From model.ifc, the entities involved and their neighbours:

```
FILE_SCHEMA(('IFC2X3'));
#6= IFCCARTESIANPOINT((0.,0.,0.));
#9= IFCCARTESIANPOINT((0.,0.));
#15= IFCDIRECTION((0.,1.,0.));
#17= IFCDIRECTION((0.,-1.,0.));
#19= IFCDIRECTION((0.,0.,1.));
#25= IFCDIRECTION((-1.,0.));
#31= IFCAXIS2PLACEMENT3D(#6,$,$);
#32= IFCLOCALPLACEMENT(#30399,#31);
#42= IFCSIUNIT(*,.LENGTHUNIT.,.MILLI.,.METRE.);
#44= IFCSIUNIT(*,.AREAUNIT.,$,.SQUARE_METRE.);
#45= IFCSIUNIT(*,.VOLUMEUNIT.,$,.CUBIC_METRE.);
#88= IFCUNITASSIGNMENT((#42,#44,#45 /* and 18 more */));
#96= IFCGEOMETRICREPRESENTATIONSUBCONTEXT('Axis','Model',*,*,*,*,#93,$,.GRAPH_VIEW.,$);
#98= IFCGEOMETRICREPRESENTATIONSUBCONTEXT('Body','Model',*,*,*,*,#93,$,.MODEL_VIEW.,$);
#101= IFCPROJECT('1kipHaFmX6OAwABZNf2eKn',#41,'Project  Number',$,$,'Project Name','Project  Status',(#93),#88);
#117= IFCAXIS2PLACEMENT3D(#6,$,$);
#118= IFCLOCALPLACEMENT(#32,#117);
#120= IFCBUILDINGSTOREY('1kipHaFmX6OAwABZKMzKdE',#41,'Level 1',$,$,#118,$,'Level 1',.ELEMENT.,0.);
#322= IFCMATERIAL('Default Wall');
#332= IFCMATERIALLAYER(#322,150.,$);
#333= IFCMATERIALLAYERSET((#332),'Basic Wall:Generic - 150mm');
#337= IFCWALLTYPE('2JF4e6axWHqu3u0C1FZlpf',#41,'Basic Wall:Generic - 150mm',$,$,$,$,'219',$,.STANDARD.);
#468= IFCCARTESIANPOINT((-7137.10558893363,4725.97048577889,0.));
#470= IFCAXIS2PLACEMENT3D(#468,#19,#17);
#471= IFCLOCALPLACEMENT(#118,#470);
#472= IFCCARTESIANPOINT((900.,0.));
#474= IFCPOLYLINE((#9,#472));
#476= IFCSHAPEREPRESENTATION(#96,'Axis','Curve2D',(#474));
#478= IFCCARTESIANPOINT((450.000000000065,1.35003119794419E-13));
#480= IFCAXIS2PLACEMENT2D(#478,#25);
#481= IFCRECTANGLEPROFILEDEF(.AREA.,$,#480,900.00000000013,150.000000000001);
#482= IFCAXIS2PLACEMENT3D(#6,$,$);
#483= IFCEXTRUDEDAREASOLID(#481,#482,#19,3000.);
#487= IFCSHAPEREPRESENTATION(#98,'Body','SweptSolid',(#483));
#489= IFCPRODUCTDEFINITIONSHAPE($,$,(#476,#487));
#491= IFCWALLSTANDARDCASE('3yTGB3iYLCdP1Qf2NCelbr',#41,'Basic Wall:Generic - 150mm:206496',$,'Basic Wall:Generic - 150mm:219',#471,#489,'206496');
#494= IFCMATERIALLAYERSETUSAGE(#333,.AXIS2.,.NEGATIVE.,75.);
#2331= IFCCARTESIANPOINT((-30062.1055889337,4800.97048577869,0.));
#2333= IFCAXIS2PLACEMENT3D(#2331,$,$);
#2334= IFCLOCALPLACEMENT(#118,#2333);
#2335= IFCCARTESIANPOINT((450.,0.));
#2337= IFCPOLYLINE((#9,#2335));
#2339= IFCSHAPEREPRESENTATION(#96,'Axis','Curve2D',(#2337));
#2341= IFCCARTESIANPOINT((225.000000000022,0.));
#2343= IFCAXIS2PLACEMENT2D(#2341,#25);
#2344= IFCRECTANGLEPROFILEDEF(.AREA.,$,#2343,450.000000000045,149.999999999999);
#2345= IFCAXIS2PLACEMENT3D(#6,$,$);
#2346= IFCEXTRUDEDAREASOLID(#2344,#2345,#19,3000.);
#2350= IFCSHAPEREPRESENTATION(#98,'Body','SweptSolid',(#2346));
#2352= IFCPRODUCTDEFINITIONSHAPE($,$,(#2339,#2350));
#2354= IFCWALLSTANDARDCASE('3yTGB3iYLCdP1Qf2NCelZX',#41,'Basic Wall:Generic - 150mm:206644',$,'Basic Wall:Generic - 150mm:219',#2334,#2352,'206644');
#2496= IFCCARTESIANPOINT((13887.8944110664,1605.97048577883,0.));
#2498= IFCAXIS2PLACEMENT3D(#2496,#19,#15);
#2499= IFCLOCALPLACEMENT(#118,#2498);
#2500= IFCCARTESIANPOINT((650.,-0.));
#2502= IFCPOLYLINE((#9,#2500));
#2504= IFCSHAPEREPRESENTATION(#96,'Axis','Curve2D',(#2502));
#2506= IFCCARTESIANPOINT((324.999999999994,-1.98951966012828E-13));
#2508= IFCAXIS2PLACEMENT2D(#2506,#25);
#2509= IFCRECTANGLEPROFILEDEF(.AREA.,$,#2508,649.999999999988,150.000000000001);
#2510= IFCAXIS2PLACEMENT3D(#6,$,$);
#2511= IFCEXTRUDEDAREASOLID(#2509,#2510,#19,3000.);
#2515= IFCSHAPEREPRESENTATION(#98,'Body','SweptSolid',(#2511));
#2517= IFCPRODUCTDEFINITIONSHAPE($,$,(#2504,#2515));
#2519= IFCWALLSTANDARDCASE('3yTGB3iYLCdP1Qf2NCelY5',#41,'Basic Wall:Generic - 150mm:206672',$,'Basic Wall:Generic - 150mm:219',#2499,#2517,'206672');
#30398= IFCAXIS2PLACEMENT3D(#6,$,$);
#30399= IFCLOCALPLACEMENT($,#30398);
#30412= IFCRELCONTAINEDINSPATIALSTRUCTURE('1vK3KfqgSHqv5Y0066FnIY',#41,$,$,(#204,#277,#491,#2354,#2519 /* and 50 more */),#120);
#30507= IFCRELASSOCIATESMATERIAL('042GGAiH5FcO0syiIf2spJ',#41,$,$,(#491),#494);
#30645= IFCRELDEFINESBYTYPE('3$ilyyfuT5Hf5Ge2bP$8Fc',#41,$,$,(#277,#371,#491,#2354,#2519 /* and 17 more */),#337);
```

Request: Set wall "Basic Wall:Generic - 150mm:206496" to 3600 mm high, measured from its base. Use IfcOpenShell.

```python
import ifcopenshell
import ifcopenshell.geom
import ifcopenshell.util.representation
import ifcopenshell.util.shape

model = ifcopenshell.open("model.ifc")
settings = ifcopenshell.geom.settings()


def volume(element):
    """Net volume in cubic metres, openings subtracted."""
    shape = ifcopenshell.geom.create_shape(settings, element)
    return ifcopenshell.util.shape.get_volume(shape.geometry)


wall = model.by_guid("3yTGB3iYLCdP1Qf2NCelbr")
before = volume(wall)

body = ifcopenshell.util.representation.get_representation(wall, "Model", "Body")
solid = body.Items[0]
old_height = solid.Depth
solid.Depth = 3600.0
after = volume(wall)

print(f"height {old_height:g} -> {solid.Depth:g}, volume {before:.3f} -> {after:.3f} m3")

model.write("model_rev.ifc")
```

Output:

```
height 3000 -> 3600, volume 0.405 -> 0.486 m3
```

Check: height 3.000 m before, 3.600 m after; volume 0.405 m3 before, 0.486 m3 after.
